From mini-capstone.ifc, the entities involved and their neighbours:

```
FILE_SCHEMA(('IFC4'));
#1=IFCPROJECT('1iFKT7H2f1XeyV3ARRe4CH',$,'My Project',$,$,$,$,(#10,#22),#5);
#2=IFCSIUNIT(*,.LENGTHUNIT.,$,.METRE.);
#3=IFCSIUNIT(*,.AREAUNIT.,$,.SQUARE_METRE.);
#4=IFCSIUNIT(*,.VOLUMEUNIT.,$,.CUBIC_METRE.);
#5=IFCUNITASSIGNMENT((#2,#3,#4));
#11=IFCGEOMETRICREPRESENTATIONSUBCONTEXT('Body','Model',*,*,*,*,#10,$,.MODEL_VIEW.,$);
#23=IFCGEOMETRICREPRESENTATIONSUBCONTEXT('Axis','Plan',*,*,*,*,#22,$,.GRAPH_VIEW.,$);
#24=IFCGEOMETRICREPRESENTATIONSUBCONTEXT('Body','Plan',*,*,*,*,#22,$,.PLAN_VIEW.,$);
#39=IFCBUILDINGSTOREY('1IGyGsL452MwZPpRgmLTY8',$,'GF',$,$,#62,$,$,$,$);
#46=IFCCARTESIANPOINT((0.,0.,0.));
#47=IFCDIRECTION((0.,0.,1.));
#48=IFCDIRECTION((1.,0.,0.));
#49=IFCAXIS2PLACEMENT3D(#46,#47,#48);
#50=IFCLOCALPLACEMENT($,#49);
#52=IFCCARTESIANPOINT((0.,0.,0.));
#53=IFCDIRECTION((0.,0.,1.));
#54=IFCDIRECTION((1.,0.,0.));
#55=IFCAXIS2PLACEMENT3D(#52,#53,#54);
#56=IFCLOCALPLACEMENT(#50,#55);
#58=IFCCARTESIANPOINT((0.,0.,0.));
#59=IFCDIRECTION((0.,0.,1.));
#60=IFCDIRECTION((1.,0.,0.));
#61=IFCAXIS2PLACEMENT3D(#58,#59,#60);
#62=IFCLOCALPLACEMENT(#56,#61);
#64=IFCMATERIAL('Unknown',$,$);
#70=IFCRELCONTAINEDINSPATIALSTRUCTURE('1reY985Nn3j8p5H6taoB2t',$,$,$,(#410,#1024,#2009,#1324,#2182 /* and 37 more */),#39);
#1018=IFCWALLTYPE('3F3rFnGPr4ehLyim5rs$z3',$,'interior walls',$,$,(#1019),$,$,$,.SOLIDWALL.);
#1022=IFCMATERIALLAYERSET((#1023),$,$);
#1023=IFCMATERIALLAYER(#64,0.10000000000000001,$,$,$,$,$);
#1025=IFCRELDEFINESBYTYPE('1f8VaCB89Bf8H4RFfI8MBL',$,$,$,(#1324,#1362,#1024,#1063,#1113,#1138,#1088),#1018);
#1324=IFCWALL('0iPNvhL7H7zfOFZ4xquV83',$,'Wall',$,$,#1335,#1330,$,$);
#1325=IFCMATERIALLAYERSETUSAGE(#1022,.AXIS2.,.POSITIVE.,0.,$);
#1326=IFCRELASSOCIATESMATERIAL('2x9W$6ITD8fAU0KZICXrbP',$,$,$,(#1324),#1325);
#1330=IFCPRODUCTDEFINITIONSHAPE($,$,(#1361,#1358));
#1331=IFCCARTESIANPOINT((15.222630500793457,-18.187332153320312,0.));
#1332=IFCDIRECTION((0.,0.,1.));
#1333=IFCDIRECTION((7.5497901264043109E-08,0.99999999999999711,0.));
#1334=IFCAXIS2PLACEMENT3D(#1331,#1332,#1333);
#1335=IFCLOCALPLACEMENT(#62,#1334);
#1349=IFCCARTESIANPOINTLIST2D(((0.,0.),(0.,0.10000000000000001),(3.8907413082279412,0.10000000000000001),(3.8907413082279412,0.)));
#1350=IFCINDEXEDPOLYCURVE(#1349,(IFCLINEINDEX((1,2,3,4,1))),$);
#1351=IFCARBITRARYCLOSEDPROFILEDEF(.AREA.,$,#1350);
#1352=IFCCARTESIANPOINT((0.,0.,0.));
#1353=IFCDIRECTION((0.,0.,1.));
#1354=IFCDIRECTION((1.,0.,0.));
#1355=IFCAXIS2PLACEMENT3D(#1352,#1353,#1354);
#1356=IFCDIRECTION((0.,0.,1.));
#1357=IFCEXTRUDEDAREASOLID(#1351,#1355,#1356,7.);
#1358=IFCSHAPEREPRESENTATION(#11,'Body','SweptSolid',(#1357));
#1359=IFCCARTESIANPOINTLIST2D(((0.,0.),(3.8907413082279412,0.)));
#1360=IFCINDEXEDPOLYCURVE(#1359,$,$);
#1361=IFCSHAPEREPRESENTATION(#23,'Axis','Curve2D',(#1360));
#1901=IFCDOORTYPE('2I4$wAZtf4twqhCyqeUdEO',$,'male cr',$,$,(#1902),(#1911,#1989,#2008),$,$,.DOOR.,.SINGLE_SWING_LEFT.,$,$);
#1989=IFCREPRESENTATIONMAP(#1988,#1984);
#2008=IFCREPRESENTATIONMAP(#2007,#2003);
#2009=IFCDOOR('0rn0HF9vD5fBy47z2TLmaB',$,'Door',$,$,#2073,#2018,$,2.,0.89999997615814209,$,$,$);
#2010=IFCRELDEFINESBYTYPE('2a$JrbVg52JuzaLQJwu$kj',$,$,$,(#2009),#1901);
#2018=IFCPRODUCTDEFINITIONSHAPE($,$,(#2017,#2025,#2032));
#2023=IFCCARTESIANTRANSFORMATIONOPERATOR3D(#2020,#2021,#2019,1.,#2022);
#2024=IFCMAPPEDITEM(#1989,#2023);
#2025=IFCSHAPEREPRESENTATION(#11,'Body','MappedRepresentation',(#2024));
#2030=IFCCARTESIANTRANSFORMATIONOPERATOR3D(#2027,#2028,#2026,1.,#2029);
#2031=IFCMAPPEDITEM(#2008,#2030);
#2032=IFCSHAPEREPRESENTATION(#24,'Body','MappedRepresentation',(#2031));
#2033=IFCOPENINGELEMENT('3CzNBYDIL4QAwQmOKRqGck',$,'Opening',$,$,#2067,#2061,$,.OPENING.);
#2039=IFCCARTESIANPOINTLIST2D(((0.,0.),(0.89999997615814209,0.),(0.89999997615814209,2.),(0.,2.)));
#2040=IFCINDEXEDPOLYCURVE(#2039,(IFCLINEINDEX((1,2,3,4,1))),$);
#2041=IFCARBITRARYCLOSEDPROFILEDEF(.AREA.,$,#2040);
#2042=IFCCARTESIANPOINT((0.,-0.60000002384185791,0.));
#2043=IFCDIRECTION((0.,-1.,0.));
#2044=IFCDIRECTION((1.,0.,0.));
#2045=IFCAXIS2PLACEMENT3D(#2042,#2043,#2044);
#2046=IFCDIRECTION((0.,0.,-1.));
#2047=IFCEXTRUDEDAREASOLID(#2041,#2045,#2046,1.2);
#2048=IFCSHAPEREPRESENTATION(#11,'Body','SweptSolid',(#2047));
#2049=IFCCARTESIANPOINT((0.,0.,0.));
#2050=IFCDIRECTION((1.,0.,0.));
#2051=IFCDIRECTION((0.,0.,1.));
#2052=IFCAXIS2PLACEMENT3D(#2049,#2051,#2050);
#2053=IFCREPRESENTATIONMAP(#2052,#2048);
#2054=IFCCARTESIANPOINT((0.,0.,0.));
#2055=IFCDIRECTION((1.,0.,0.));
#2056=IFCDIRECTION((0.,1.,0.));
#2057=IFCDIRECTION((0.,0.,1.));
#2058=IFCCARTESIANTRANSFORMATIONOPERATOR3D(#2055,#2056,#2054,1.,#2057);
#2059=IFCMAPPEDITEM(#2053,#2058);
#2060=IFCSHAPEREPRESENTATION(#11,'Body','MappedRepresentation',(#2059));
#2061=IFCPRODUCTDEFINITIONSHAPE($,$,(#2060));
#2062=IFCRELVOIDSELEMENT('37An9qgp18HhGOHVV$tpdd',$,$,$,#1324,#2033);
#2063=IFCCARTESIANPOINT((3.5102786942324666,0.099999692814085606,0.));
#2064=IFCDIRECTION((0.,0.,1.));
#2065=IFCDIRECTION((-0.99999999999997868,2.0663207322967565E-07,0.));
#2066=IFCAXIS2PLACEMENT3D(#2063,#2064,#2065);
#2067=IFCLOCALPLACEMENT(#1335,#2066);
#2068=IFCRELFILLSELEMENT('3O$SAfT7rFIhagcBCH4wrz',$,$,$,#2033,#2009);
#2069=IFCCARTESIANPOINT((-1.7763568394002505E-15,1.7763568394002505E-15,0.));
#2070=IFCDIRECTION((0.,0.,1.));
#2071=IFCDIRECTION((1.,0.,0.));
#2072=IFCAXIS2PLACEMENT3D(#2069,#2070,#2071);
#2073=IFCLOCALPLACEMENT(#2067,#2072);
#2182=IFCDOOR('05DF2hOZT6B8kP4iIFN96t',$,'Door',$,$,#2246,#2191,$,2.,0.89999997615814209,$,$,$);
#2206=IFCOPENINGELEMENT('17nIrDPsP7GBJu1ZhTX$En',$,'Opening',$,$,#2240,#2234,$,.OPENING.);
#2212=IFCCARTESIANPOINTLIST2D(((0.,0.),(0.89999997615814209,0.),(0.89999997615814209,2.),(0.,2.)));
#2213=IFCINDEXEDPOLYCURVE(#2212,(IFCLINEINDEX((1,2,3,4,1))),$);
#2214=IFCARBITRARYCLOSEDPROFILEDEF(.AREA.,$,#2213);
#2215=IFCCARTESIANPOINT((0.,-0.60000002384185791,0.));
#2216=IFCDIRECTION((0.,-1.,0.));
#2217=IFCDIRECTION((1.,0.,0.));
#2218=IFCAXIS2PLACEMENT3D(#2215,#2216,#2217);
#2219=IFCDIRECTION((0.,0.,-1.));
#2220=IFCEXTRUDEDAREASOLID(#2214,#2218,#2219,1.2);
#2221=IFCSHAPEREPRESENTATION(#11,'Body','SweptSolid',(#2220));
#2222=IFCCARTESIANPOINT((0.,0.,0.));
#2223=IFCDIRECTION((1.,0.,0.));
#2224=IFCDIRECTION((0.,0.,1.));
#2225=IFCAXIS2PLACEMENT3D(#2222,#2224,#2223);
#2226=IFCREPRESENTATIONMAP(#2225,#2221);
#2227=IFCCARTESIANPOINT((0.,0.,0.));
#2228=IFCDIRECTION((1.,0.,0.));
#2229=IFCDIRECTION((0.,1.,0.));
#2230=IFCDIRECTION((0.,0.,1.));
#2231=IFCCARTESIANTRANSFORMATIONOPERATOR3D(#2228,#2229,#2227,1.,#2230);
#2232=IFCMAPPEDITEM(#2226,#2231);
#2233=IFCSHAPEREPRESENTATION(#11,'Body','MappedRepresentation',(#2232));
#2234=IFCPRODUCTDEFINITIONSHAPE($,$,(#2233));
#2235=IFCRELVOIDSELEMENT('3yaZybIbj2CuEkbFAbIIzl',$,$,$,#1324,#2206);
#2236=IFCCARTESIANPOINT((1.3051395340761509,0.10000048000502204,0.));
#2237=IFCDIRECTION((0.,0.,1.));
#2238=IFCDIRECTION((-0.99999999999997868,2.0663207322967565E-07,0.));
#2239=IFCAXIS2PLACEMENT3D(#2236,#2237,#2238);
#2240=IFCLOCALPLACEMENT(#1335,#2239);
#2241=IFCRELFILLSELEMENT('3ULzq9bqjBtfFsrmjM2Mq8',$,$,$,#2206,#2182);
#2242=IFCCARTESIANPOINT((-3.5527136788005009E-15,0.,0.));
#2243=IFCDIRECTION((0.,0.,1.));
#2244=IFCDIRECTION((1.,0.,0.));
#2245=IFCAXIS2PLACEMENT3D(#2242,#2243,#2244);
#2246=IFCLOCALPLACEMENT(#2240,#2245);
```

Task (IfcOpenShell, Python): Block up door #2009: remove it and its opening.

```python
import ifcopenshell
import ifcopenshell.api.feature
import ifcopenshell.api.root
import ifcopenshell.geom
import ifcopenshell.util.shape

model = ifcopenshell.open("mini-capstone.ifc")
settings = ifcopenshell.geom.settings()


def volume(element):
    """Net volume in cubic metres, openings subtracted."""
    shape = ifcopenshell.geom.create_shape(settings, element)
    return ifcopenshell.util.shape.get_volume(shape.geometry)


door = model.by_id(2009)
opening = door.FillsVoids[0].RelatingOpeningElement
wall = opening.VoidsElements[0].RelatingBuildingElement
before = volume(wall)

ifcopenshell.api.root.remove_product(model, product=door)
ifcopenshell.api.feature.remove_feature(model, feature=opening)

after = volume(wall)

print(f"wall volume {before:.3f} -> {after:.3f} m3")

model.write("mini-capstone_edited.ifc")
```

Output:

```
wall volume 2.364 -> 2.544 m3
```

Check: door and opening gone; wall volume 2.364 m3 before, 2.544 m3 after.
